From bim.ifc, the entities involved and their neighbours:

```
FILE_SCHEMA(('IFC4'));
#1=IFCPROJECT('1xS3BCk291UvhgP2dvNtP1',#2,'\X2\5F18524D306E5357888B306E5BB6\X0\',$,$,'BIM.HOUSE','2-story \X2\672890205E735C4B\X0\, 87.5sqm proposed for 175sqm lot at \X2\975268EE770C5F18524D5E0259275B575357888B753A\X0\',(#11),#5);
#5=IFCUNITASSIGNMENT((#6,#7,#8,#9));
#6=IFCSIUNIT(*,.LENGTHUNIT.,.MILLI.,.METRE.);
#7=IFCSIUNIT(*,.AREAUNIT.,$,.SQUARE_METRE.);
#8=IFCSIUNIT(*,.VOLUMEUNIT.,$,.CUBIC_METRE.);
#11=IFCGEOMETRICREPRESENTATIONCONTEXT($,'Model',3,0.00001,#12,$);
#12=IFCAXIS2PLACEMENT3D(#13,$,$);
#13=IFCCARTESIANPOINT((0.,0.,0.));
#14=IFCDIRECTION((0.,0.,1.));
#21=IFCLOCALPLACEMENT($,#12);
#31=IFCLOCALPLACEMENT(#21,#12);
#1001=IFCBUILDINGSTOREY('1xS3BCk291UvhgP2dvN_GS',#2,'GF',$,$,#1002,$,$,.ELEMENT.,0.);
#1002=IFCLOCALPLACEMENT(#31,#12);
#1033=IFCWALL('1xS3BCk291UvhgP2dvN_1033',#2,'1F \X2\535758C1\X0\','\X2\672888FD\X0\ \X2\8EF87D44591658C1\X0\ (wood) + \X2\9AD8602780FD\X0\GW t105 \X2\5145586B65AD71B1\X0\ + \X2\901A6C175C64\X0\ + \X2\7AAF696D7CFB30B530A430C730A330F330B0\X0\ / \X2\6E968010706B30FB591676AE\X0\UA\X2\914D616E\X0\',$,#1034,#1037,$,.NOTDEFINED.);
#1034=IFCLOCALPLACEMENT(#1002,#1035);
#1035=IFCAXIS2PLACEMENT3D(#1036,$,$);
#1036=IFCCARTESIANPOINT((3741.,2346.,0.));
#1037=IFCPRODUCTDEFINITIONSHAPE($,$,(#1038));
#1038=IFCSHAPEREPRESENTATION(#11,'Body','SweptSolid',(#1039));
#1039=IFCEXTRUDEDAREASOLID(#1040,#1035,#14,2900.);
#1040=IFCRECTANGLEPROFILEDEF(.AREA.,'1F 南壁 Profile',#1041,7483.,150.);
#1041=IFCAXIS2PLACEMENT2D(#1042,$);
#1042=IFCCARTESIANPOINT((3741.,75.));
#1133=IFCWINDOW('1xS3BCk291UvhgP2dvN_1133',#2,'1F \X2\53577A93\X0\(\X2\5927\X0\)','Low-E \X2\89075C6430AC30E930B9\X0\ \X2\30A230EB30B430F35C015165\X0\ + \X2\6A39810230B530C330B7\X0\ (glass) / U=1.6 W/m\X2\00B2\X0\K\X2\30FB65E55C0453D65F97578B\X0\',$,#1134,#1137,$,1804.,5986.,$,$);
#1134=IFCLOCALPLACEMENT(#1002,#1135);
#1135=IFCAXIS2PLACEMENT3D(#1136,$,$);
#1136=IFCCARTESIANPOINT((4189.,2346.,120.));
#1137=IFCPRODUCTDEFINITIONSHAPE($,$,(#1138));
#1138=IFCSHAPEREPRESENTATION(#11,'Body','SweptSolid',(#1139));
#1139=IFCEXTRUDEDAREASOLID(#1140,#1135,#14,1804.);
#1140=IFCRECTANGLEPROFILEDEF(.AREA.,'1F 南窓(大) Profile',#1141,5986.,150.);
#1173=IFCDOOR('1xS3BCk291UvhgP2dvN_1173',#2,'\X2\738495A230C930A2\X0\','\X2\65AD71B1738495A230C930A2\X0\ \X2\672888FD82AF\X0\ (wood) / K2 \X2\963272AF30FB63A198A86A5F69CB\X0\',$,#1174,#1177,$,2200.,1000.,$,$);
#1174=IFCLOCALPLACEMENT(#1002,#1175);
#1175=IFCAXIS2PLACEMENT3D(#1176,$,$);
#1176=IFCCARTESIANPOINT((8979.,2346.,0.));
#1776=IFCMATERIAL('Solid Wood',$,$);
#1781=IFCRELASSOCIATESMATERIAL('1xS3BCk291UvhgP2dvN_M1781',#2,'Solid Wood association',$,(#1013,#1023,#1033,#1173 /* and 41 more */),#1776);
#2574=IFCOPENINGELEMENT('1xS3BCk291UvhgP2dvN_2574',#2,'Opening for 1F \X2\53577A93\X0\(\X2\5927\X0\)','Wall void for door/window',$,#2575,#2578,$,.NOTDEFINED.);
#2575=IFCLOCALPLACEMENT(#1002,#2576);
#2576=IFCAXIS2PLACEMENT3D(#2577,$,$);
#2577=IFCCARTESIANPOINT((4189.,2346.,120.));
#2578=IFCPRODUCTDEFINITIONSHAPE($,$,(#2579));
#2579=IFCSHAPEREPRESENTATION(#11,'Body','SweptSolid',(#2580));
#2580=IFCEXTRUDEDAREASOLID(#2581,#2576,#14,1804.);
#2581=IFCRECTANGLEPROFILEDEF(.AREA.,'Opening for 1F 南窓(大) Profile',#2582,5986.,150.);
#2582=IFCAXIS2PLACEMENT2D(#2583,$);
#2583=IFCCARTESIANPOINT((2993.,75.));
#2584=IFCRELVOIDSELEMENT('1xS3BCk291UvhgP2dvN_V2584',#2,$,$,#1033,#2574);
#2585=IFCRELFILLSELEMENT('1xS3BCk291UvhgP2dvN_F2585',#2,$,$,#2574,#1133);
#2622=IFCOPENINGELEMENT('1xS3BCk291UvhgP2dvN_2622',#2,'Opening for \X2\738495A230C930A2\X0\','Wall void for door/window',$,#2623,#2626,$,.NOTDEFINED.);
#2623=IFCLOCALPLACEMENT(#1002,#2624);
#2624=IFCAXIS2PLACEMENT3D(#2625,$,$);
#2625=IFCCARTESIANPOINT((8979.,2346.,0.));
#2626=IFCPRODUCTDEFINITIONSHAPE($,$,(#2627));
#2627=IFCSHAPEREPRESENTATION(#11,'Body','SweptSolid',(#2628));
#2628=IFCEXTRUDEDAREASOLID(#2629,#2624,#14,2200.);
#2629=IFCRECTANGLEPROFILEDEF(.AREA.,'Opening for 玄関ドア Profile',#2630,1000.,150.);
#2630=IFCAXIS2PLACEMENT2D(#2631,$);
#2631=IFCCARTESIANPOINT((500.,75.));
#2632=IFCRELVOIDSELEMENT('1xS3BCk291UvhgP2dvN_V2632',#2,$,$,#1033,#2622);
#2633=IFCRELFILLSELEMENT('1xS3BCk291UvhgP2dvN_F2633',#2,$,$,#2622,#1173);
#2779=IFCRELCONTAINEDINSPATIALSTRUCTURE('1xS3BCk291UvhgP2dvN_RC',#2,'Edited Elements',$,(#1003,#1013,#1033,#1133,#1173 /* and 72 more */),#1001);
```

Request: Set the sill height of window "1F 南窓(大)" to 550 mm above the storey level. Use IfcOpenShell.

```python
import numpy as np
import ifcopenshell
import ifcopenshell.api.geometry
import ifcopenshell.geom
import ifcopenshell.util.element
import ifcopenshell.util.placement
import ifcopenshell.util.shape
import ifcopenshell.util.unit

model = ifcopenshell.open("bim.ifc")
unit_scale = ifcopenshell.util.unit.calculate_unit_scale(model)

window = model.by_guid("1xS3BCk291UvhgP2dvN_1133")
opening = window.FillsVoids[0].RelatingOpeningElement
storey = ifcopenshell.util.element.get_container(window, ifc_class="IfcBuildingStorey")
level = ifcopenshell.util.placement.get_local_placement(storey.ObjectPlacement)[2, 3]

# The opening's origin need not be at the sill, so measure its lowest point.
shape = ifcopenshell.geom.create_shape(ifcopenshell.geom.settings(), opening)
bottom = ifcopenshell.util.shape.get_shape_bottom_elevation(shape, shape.geometry) / unit_scale
dz = level + 0.55 / unit_scale - bottom

shift = np.array([0.0, 0.0, dz])
# The window is not placed relative to its opening, so move both.
for product in (opening, window):
    matrix = ifcopenshell.util.placement.get_local_placement(product.ObjectPlacement)
    matrix[:3, 3] += shift
    ifcopenshell.api.geometry.edit_object_placement(model, product=product, matrix=matrix, is_si=False)

print(f"moved by {dz * unit_scale:+.3f} m")

model.write("bim_rev.ifc")
```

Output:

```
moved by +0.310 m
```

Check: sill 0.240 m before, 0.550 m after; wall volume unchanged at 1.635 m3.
